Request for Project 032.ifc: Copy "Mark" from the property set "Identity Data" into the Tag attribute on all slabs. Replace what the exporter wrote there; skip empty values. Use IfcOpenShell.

First a look at what the model holds.

```python
import ifcopenshell
import ifcopenshell.util.element

model = ifcopenshell.open("Project 032.ifc")
print(model.schema)
slabs = model.by_type("IfcSlab")
print(len(slabs), "slabs")
for e in slabs[:8]:
    source = ifcopenshell.util.element.get_pset(e, "Identity Data", "Mark")
    target = e.Tag
    print(e.id(), repr(source), repr(target), sep=" | ")
```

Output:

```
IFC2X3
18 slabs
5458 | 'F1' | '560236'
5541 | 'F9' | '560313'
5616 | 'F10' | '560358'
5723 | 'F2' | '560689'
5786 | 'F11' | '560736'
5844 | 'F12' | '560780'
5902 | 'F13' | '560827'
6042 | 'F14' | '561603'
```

```python
import ifcopenshell
import ifcopenshell.util.element

model = ifcopenshell.open("Project 032.ifc")

count = 0
for e in model.by_type("IfcSlab"):
    value = ifcopenshell.util.element.get_pset(e, "Identity Data", "Mark")
    current = e.Tag
    if not value or not value.strip() or current == value:
        continue
    e.Tag = value
    count += 1

print(count, "slabs updated")

model.write("Project 032_rev.ifc")
```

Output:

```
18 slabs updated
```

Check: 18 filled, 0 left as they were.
